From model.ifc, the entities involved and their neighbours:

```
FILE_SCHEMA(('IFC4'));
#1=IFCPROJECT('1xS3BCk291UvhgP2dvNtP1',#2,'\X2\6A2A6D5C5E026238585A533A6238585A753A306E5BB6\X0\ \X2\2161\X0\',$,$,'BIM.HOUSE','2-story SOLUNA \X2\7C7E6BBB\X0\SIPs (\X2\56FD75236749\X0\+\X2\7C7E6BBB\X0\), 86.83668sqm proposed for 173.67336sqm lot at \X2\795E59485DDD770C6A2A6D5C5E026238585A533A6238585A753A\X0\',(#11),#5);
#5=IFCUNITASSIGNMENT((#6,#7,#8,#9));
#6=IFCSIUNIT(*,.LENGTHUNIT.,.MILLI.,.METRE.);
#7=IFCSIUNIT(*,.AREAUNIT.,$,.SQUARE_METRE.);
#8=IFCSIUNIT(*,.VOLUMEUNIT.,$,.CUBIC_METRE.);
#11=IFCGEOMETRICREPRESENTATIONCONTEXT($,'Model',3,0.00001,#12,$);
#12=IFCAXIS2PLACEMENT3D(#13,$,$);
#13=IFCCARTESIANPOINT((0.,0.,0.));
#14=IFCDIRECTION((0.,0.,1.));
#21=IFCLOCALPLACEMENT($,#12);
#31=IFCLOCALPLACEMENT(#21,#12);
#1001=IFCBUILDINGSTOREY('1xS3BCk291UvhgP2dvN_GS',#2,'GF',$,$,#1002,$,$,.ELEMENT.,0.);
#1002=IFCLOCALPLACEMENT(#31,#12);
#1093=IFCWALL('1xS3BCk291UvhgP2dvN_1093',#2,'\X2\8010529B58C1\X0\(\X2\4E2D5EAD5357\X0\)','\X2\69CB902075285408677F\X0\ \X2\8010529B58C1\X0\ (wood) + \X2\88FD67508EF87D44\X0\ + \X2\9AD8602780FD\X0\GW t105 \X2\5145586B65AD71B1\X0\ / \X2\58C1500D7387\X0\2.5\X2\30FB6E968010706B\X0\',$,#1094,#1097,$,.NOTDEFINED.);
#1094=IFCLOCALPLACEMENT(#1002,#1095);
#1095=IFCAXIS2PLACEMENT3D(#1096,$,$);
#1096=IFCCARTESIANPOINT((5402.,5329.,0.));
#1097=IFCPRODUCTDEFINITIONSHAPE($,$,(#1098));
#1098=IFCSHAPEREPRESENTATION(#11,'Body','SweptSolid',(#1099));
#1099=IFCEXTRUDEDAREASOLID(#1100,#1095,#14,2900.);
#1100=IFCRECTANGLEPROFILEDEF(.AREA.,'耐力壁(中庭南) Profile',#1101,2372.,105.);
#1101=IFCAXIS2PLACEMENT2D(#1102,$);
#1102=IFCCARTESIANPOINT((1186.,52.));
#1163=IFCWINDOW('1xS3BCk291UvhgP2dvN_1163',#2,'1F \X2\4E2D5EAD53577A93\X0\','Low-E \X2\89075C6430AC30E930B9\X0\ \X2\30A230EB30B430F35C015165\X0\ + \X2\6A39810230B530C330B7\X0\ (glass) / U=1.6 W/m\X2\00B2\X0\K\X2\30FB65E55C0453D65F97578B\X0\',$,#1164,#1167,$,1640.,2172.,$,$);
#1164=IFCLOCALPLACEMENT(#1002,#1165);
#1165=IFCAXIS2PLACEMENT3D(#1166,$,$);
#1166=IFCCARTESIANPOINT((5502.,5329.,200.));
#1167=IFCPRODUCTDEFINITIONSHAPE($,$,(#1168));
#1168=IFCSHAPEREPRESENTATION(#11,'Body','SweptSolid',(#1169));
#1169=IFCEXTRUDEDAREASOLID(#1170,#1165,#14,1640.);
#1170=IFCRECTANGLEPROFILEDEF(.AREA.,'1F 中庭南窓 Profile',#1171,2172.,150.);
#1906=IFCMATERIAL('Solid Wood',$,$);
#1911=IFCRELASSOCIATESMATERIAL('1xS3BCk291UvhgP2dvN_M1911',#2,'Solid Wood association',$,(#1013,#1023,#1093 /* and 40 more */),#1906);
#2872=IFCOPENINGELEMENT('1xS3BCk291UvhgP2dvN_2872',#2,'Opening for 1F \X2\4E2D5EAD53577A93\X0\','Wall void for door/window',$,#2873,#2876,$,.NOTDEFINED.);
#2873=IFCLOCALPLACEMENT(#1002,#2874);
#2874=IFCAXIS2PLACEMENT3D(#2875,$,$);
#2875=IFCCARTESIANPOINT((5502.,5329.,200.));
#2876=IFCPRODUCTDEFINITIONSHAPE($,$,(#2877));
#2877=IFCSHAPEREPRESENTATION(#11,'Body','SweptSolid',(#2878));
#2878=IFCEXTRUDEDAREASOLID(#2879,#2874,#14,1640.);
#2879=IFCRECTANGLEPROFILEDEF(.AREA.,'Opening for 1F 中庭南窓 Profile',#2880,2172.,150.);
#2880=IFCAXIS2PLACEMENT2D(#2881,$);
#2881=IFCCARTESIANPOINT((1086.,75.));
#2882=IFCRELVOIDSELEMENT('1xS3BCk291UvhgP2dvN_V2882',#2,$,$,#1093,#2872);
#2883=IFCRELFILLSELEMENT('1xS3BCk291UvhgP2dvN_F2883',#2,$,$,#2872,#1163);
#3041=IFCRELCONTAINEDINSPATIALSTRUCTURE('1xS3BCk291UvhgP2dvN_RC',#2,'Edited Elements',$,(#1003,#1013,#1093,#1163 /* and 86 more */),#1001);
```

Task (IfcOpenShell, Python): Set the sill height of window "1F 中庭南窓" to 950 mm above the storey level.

```python
import numpy as np
import ifcopenshell
import ifcopenshell.api.geometry
import ifcopenshell.geom
import ifcopenshell.util.element
import ifcopenshell.util.placement
import ifcopenshell.util.shape
import ifcopenshell.util.unit

model = ifcopenshell.open("model.ifc")
unit_scale = ifcopenshell.util.unit.calculate_unit_scale(model)

window = model.by_guid("1xS3BCk291UvhgP2dvN_1163")
opening = window.FillsVoids[0].RelatingOpeningElement
storey = ifcopenshell.util.element.get_container(window, ifc_class="IfcBuildingStorey")
level = ifcopenshell.util.placement.get_local_placement(storey.ObjectPlacement)[2, 3]

# The opening's origin need not be at the sill, so measure its lowest point.
shape = ifcopenshell.geom.create_shape(ifcopenshell.geom.settings(), opening)
bottom = ifcopenshell.util.shape.get_shape_bottom_elevation(shape, shape.geometry) / unit_scale
dz = level + 950.0 - bottom

shift = np.array([0.0, 0.0, dz])
# The window is not placed relative to its opening, so move both.
for product in (opening, window):
    matrix = ifcopenshell.util.placement.get_local_placement(product.ObjectPlacement)
    matrix[:3, 3] += shift
    ifcopenshell.api.geometry.edit_object_placement(model, product=product, matrix=matrix, is_si=False)

print(f"moved by {dz * unit_scale:+.3f} m")

model.write("model_rev.ifc")
```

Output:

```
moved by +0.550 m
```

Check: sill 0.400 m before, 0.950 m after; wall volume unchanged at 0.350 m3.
